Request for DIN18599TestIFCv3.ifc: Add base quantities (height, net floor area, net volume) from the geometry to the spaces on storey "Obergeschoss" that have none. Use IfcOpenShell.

First a look at what the model holds.

```python
import ifcopenshell
import ifcopenshell.util.element
import ifcopenshell.util.unit

model = ifcopenshell.open("DIN18599TestIFCv3.ifc")
print(model.schema)
for unit_type in ("LENGTHUNIT", "AREAUNIT", "VOLUMEUNIT"):
    print(unit_type, ifcopenshell.util.unit.calculate_unit_scale(model, unit_type))
storey = next(s for s in model.by_type("IfcBuildingStorey") if s.Name == "Obergeschoss")
spaces = [e for e in ifcopenshell.util.element.get_decomposition(storey) if e.is_a("IfcSpace")]
for e in sorted(spaces, key=lambda e: e.id()):
    print(e.id(), e.is_a(), e.Name, list(ifcopenshell.util.element.get_psets(e, qtos_only=True)), sep=" | ")
```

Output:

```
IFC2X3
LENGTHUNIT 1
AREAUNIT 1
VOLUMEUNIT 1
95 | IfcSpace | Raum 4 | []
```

```python
import ifcopenshell
import ifcopenshell.api.pset
import ifcopenshell.geom
import ifcopenshell.util.element
import ifcopenshell.util.shape
import ifcopenshell.util.unit

model = ifcopenshell.open("DIN18599TestIFCv3.ifc")
unit_scale = ifcopenshell.util.unit.calculate_unit_scale(model)
area_scale = ifcopenshell.util.unit.calculate_unit_scale(model, "AREAUNIT")
volume_scale = ifcopenshell.util.unit.calculate_unit_scale(model, "VOLUMEUNIT")
settings = ifcopenshell.geom.settings()

storey = next(s for s in model.by_type("IfcBuildingStorey") if s.Name == "Obergeschoss")
spaces = [e for e in ifcopenshell.util.element.get_decomposition(storey) if e.is_a("IfcSpace")]

for e in sorted(spaces, key=lambda e: e.id()):
    if ifcopenshell.util.element.get_psets(e, qtos_only=True, should_inherit=False):
        continue
    # Geometry comes back in metres, in the element's own axes.
    shape = ifcopenshell.geom.create_shape(settings, e)
    values = {
        "Height": ifcopenshell.util.shape.get_z(shape.geometry) / unit_scale,
        "NetFloorArea": ifcopenshell.util.shape.get_footprint_area(shape.geometry) / area_scale,
        "NetVolume": ifcopenshell.util.shape.get_volume(shape.geometry) / volume_scale,
    }
    qto = ifcopenshell.api.pset.add_qto(model, product=e, name="BaseQuantities")
    ifcopenshell.api.pset.edit_qto(model, qto=qto, properties=values)
    print(e.id(), {k: round(v, 3) for k, v in values.items()})

model.write("DIN18599TestIFCv3_edited.ifc")
```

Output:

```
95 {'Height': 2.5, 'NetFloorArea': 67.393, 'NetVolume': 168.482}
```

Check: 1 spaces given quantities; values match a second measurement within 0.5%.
